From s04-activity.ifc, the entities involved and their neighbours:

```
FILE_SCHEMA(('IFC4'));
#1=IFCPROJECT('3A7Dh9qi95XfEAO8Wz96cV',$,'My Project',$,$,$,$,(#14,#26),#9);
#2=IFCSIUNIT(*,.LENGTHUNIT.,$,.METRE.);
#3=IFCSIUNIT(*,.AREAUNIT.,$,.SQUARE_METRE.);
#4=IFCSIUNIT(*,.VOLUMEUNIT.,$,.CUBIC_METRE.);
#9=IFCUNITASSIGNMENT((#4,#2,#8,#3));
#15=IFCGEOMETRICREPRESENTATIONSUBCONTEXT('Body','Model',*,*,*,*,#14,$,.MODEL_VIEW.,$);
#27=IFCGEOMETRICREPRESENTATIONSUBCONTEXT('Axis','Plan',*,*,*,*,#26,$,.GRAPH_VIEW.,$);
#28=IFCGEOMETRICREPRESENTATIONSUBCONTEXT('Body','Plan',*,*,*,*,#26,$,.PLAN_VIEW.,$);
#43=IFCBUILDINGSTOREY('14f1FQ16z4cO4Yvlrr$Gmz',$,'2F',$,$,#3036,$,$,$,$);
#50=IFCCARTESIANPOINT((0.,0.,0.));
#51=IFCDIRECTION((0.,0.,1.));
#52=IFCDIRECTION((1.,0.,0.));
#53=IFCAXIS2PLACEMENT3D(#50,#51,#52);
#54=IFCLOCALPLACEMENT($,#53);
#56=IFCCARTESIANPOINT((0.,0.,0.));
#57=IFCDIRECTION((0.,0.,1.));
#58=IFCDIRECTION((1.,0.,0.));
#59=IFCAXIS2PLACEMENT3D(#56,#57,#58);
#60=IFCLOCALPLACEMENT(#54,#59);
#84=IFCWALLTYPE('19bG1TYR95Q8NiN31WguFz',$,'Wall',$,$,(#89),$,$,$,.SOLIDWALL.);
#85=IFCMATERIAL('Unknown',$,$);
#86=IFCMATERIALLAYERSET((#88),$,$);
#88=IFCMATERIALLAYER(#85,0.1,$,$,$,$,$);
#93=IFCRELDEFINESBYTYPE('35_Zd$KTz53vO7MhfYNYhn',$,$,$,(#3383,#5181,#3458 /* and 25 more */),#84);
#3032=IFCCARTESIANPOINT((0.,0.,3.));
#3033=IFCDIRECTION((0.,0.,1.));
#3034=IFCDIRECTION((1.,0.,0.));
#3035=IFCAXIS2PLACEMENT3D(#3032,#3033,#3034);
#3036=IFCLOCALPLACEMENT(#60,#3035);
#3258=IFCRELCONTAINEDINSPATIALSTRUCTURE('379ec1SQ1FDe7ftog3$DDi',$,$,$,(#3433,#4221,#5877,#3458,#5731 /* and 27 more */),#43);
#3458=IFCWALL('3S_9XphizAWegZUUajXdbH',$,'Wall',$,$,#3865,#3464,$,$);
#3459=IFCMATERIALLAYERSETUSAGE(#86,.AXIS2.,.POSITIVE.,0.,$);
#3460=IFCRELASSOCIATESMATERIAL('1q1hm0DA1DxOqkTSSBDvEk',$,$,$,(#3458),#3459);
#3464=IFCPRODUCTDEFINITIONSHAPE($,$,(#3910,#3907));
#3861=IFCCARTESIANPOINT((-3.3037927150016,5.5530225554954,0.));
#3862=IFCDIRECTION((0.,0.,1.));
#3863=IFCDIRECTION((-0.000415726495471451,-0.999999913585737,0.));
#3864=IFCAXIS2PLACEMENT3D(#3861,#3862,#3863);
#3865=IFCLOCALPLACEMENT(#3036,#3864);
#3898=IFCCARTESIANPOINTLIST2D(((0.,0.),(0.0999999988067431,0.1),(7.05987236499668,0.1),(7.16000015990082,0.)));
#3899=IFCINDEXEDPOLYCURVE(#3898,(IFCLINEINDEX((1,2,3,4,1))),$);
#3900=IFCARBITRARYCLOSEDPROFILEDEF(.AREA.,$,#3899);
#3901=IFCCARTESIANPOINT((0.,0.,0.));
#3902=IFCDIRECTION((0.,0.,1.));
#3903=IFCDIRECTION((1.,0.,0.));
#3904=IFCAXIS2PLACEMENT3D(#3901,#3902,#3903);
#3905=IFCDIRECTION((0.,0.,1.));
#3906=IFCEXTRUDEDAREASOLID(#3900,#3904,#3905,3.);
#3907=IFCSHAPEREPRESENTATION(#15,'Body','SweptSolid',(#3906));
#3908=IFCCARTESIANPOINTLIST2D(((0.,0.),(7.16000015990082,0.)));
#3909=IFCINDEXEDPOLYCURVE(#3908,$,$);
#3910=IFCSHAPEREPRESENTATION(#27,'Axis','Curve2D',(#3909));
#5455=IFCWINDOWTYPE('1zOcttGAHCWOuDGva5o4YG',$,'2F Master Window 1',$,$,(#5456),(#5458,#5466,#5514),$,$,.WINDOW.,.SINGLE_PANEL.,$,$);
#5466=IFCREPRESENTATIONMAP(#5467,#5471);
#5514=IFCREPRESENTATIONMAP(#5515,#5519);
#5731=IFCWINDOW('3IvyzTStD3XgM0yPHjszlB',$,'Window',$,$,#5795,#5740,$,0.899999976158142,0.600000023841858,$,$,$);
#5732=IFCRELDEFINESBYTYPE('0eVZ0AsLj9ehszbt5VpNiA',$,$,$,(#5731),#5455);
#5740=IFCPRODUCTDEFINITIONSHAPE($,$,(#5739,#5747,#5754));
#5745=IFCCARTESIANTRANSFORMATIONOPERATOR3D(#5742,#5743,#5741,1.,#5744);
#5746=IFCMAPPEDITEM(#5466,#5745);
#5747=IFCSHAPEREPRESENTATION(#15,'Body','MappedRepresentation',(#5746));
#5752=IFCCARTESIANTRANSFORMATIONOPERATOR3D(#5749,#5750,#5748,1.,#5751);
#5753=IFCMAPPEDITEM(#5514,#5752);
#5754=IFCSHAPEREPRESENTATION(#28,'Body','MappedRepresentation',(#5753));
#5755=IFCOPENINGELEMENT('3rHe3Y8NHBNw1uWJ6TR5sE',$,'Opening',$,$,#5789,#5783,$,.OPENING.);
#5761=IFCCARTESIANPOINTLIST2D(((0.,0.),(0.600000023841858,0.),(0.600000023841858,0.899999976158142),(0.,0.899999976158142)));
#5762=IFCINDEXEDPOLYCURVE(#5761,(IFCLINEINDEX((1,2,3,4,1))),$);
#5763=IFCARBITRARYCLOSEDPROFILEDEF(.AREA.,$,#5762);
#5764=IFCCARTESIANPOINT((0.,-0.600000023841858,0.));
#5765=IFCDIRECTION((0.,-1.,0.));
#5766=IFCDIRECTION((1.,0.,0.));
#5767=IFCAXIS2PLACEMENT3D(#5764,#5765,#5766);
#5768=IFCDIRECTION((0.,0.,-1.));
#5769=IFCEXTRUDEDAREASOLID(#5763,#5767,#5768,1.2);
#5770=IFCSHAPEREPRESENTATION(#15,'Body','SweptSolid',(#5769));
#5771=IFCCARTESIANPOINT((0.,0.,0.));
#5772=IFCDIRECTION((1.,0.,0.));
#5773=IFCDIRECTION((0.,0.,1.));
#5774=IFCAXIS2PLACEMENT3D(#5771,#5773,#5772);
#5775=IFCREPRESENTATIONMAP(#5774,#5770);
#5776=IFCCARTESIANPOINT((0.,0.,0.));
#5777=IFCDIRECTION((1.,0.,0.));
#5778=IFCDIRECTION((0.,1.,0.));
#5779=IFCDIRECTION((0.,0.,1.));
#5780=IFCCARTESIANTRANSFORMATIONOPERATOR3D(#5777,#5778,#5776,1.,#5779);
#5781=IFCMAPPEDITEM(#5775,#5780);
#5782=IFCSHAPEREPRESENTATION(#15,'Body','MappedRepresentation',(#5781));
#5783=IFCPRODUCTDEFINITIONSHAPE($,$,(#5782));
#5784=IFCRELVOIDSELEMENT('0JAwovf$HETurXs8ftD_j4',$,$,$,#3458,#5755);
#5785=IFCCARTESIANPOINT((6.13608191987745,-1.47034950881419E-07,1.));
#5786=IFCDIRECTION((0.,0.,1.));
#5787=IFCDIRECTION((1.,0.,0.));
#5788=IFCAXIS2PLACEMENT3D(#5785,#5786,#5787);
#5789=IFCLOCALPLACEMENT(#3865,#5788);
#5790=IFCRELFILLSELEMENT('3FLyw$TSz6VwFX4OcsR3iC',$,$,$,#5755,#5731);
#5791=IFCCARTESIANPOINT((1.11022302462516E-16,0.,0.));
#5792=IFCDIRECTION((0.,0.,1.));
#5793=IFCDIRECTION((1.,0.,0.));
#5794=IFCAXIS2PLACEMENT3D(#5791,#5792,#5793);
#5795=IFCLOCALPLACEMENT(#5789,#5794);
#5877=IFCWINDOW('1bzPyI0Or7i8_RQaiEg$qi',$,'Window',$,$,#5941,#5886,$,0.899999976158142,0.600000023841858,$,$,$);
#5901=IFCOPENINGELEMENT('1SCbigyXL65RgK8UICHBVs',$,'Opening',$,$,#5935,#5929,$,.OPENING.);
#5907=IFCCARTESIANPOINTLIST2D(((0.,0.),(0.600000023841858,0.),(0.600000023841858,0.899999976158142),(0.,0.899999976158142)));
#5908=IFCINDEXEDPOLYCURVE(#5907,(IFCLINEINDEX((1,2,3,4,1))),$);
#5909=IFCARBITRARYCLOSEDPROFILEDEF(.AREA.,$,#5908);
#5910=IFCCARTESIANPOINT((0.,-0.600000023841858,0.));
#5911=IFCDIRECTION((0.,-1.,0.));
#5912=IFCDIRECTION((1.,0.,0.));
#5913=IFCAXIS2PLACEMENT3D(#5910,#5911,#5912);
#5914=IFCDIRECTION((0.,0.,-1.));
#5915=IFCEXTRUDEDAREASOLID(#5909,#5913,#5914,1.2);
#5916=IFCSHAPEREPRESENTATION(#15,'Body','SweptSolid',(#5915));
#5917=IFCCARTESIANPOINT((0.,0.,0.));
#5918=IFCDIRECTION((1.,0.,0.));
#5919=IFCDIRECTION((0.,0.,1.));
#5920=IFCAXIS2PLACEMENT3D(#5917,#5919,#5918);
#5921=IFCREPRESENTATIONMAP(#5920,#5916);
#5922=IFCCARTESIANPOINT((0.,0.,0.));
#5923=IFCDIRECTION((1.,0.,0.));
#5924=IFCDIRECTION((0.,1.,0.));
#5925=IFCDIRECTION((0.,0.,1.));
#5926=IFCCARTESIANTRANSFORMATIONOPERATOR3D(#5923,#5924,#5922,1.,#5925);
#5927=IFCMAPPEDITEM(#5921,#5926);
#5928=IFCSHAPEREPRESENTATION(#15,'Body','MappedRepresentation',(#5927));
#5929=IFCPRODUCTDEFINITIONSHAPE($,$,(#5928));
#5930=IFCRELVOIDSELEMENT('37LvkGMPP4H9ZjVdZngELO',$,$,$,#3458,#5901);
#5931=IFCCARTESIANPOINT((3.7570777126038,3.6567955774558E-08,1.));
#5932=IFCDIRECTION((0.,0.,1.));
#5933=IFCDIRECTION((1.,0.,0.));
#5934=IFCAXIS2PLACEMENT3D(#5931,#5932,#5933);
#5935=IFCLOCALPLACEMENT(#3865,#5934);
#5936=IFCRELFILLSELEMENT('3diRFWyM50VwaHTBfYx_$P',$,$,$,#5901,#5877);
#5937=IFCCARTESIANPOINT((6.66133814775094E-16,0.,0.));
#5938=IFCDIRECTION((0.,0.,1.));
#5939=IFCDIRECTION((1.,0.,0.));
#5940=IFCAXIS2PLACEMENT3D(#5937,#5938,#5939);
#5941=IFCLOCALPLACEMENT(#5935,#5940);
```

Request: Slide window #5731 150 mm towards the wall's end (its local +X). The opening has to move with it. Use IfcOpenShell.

```python
import ifcopenshell
import ifcopenshell.api.geometry
import ifcopenshell.util.placement
import ifcopenshell.util.unit

model = ifcopenshell.open("s04-activity.ifc")
unit_scale = ifcopenshell.util.unit.calculate_unit_scale(model)

window = model.by_guid("3IvyzTStD3XgM0yPHjszlB")
opening = window.FillsVoids[0].RelatingOpeningElement
wall = opening.VoidsElements[0].RelatingBuildingElement

wall_matrix = ifcopenshell.util.placement.get_local_placement(wall.ObjectPlacement)
shift = wall_matrix[:3, 0] * 0.15 / unit_scale
before = ifcopenshell.util.placement.get_local_placement(window.ObjectPlacement)[:3, 3].copy()

# The window is placed relative to its opening, so it follows when the opening moves.
matrix = ifcopenshell.util.placement.get_local_placement(opening.ObjectPlacement)
matrix[:3, 3] += shift
ifcopenshell.api.geometry.edit_object_placement(
    model, product=opening, matrix=matrix, is_si=False, should_transform_children=True
)

after = ifcopenshell.util.placement.get_local_placement(window.ObjectPlacement)[:3, 3]
print("window moved by", (after - before).round(3) + 0.0)

model.write("s04-activity_updated.ifc")
```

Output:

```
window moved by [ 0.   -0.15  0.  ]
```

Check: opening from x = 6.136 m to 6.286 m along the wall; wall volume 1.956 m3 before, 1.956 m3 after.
